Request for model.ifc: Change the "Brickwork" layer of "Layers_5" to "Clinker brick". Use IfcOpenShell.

First a look at what the model holds.

```python
import ifcopenshell
import ifcopenshell.util.element

model = ifcopenshell.open("model.ifc")
print(model.schema)
for layer_set in model.by_type("IfcMaterialLayerSet"):
    if layer_set.LayerSetName == "Layers_5":
        for layer in layer_set.MaterialLayers:
            print(layer.id(), layer.Material and layer.Material.Name, layer.LayerThickness, sep=" | ")
        print(len(ifcopenshell.util.element.get_elements_by_material(model, layer_set)), "elements and types use it")
print(sorted(m.Name for m in model.by_type("IfcMaterial") if m.Name)[:60])
```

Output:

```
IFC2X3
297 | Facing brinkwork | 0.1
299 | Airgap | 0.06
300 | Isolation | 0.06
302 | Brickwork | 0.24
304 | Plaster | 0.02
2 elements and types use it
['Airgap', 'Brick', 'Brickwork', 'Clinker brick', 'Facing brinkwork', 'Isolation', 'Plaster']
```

```python
import ifcopenshell
import ifcopenshell.api.material

model = ifcopenshell.open("model.ifc")

layer_set = next(s for s in model.by_type("IfcMaterialLayerSet") if s.LayerSetName == "Layers_5")
layer = next(l for l in layer_set.MaterialLayers if l.Material and l.Material.Name == "Brickwork")
material = next(m for m in model.by_type("IfcMaterial") if m.Name == "Clinker brick")

# Point this one layer at the other material; renaming the old one would change it everywhere.
ifcopenshell.api.material.edit_layer(model, layer=layer, attributes={}, material=material)

print([l.Material.Name if l.Material else None for l in layer_set.MaterialLayers])

model.write("model_edited.ifc")
```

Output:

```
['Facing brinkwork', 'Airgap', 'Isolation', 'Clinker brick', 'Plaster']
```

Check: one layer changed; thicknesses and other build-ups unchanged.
